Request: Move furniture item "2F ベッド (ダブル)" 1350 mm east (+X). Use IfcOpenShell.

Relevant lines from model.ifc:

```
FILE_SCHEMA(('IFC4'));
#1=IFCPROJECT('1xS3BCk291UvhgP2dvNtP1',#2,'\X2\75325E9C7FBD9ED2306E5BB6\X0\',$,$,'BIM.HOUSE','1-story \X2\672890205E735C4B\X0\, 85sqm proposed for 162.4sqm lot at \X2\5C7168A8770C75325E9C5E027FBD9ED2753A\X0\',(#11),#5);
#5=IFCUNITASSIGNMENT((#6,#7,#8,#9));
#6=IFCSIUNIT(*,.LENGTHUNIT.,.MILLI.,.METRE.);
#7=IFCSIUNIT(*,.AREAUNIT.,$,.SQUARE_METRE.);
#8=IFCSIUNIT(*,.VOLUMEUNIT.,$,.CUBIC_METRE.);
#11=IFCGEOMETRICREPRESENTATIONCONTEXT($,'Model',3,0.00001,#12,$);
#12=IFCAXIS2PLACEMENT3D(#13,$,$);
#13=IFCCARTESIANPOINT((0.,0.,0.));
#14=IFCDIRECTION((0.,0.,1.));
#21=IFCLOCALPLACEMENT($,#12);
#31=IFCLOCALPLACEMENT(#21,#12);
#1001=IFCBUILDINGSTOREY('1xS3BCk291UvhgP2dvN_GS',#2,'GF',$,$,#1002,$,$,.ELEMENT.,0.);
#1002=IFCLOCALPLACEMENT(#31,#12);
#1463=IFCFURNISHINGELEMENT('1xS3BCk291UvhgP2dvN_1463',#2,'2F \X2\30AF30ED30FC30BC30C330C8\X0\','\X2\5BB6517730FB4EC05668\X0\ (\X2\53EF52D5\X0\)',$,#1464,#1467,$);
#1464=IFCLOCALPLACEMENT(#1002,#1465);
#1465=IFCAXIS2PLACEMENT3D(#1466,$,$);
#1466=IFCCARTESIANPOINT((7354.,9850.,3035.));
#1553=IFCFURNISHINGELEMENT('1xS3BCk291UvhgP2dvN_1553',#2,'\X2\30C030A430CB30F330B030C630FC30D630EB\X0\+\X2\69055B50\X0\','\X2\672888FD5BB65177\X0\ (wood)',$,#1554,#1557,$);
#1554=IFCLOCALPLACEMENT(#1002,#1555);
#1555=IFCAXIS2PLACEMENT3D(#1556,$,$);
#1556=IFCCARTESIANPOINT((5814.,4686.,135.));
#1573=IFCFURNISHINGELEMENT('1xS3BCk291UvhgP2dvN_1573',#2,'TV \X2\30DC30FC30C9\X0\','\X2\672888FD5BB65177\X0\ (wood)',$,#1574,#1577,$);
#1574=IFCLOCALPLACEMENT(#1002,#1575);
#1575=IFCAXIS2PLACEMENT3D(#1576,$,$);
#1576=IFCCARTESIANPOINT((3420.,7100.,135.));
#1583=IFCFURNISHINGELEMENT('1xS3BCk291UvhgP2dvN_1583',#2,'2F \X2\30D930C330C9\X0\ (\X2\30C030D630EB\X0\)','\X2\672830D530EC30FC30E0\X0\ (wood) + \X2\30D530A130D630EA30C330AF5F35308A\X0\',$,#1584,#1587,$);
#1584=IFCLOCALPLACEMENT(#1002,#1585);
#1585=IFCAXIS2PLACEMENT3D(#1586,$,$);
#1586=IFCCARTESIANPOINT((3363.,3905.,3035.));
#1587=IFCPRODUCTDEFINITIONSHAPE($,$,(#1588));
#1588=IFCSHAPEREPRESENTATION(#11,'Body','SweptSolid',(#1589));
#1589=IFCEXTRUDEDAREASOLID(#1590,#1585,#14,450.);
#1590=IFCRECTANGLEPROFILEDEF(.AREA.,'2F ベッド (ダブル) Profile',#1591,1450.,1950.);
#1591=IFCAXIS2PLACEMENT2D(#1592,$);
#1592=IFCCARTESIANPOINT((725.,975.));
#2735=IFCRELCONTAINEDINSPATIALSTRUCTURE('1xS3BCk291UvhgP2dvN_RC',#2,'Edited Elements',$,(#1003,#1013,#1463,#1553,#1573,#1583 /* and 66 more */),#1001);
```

```python
import ifcopenshell
import ifcopenshell.api.geometry
import ifcopenshell.util.placement

model = ifcopenshell.open("model.ifc")

item = model.by_guid("1xS3BCk291UvhgP2dvN_1583")
matrix = ifcopenshell.util.placement.get_local_placement(item.ObjectPlacement)
matrix[0, 3] += 1350.0
ifcopenshell.api.geometry.edit_object_placement(model, product=item, matrix=matrix, is_si=False)

print(ifcopenshell.util.placement.get_local_placement(item.ObjectPlacement).round(3) + 0.0)

model.write("model_v2.ifc")
```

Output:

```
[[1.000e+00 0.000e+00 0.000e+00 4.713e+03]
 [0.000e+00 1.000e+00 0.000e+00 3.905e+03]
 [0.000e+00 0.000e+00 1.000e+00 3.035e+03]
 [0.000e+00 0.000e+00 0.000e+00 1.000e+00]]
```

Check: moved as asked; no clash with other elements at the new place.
